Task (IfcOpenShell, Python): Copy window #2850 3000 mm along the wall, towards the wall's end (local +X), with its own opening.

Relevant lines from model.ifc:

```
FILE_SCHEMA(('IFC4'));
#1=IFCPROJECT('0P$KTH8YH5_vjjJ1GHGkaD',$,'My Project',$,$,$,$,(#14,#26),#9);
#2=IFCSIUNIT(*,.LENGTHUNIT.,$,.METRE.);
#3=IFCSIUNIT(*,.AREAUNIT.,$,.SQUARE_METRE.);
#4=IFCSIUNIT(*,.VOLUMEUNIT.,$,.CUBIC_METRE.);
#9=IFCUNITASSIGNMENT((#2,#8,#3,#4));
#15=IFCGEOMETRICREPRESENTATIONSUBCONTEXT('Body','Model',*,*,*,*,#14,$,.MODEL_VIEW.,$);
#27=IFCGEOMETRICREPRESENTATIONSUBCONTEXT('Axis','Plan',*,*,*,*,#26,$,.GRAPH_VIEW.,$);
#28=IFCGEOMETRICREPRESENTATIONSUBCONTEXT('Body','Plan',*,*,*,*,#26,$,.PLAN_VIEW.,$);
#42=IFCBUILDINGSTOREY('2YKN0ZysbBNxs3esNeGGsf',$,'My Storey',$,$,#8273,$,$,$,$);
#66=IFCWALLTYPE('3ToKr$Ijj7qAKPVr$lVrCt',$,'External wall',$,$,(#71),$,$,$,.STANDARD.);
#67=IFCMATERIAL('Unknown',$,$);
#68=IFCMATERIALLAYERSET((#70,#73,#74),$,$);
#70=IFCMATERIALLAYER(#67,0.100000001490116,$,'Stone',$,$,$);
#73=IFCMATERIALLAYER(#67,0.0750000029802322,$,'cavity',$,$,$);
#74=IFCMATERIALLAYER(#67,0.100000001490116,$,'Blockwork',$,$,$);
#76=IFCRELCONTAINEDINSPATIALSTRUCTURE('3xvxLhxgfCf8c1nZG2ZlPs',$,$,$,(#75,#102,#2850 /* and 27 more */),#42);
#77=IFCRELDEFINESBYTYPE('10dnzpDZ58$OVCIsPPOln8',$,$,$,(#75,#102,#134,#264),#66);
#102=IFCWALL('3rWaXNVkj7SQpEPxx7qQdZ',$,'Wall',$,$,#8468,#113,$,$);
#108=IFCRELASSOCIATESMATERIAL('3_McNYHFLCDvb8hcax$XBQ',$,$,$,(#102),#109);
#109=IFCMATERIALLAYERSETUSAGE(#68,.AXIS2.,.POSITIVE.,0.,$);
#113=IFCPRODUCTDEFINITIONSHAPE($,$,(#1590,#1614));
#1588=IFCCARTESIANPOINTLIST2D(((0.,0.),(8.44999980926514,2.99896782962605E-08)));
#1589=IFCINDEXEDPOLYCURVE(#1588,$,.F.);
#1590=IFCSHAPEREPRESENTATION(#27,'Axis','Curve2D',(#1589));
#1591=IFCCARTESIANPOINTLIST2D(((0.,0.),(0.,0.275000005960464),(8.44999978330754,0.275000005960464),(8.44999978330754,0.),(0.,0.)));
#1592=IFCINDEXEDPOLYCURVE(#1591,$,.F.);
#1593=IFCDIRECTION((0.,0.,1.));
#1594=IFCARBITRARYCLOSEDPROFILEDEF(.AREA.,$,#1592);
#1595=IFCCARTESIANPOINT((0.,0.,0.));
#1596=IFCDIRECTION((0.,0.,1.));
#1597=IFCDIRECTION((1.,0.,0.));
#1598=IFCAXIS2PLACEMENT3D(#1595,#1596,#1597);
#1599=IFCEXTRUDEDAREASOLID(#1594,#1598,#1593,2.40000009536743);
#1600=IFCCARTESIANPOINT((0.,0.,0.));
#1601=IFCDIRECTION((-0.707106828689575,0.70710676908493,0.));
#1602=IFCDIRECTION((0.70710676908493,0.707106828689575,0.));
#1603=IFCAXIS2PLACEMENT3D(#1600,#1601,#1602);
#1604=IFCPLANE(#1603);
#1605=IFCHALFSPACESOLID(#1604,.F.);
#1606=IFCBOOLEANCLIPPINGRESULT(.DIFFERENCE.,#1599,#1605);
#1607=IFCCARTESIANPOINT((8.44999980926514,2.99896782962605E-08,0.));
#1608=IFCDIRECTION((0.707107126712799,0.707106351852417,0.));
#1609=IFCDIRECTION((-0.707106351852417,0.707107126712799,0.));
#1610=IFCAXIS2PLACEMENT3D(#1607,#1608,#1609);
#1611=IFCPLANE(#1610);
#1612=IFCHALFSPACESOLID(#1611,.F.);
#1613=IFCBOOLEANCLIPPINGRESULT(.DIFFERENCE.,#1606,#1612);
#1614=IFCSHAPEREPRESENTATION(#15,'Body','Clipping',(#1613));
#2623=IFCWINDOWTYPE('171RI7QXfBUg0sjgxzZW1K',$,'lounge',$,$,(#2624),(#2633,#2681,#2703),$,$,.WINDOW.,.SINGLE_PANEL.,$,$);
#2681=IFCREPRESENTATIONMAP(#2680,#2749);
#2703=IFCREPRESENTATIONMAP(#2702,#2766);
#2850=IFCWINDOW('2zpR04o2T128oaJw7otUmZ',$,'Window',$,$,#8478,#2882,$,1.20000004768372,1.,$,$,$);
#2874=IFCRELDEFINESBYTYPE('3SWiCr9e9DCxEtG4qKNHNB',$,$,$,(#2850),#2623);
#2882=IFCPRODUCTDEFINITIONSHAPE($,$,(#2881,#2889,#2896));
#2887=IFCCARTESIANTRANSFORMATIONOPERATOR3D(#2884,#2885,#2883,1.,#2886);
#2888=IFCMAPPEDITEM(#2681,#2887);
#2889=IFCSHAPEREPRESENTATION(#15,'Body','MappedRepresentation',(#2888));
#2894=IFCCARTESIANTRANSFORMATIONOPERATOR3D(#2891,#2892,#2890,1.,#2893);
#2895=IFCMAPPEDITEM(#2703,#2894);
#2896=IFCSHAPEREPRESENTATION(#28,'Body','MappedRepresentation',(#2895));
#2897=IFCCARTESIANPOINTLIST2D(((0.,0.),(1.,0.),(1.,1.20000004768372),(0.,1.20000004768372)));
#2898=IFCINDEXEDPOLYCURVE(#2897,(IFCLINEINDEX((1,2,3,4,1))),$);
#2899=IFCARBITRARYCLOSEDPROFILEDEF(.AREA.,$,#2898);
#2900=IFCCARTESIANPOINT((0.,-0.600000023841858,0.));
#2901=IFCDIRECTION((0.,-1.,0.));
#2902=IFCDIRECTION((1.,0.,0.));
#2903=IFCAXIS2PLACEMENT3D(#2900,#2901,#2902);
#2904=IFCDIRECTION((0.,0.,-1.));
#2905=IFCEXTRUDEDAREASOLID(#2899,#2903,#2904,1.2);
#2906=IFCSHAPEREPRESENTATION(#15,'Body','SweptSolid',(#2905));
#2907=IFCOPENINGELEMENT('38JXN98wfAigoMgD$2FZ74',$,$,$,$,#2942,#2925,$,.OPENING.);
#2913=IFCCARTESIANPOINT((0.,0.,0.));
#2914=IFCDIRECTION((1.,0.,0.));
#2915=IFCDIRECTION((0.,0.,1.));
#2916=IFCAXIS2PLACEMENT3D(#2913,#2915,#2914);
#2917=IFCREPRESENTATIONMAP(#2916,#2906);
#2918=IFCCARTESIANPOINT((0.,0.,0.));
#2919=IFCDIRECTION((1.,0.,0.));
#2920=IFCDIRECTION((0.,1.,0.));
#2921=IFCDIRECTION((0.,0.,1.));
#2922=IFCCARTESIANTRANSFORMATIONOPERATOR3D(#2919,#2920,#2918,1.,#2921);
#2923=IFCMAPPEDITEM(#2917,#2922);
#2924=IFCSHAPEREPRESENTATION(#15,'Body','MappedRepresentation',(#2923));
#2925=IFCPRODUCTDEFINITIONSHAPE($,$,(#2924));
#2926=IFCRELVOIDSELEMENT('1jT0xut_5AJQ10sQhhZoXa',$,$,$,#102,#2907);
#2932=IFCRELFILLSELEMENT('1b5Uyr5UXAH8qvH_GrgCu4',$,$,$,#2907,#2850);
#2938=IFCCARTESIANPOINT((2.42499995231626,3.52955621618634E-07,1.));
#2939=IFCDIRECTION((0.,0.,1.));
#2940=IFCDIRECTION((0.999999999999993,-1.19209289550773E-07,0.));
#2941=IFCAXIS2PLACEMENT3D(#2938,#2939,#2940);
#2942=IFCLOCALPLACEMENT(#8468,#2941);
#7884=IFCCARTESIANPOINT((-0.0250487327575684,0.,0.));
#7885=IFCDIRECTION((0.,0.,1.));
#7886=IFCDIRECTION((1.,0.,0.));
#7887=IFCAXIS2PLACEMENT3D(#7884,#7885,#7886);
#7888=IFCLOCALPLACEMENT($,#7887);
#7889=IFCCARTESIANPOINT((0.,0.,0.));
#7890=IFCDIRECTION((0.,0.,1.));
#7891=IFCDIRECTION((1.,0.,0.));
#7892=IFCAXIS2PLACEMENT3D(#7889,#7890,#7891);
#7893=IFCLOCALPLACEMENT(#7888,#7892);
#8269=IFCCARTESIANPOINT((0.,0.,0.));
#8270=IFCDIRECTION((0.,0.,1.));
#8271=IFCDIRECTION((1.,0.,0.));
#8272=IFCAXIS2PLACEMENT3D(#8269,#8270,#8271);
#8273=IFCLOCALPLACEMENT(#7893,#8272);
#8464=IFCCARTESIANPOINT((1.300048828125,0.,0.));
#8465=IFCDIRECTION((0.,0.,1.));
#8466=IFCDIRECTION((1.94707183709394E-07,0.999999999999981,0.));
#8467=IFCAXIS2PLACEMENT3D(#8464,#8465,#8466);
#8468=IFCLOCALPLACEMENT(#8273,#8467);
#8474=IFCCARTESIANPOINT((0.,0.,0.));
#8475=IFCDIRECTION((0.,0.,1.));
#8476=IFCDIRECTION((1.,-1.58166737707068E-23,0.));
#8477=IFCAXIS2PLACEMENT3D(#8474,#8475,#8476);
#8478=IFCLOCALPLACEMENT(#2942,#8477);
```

```python
import ifcopenshell
import ifcopenshell.api.feature
import ifcopenshell.api.geometry
import ifcopenshell.api.root
import ifcopenshell.geom
import ifcopenshell.util.element
import ifcopenshell.util.placement
import ifcopenshell.util.shape

model = ifcopenshell.open("model.ifc")
settings = ifcopenshell.geom.settings()


def volume(element):
    """Net volume in cubic metres, openings subtracted."""
    shape = ifcopenshell.geom.create_shape(settings, element)
    return ifcopenshell.util.shape.get_volume(shape.geometry)


window = model.by_guid("2zpR04o2T128oaJw7otUmZ")
opening = window.FillsVoids[0].RelatingOpeningElement
wall = opening.VoidsElements[0].RelatingBuildingElement
before = volume(wall)
shift = ifcopenshell.util.placement.get_local_placement(wall.ObjectPlacement)[:3, 0] * 3.0

# copy_class copies the void relationship, type, container and properties, but no geometry.
new_opening = ifcopenshell.api.root.copy_class(model, product=opening)
new_opening.Representation = ifcopenshell.util.element.copy_deep(
    model, opening.Representation, exclude=["IfcGeometricRepresentationContext", "IfcRepresentationMap"]
)
new_window = ifcopenshell.api.root.copy_class(model, product=window)
new_window.Representation = ifcopenshell.util.element.copy_deep(
    model, window.Representation, exclude=["IfcGeometricRepresentationContext", "IfcRepresentationMap"]
)
ifcopenshell.api.feature.add_filling(model, opening=new_opening, element=new_window)

for old, new in ((opening, new_opening), (window, new_window)):
    matrix = ifcopenshell.util.placement.get_local_placement(old.ObjectPlacement)
    matrix[:3, 3] += shift
    ifcopenshell.api.geometry.edit_object_placement(model, product=new, matrix=matrix, is_si=False)

after = volume(wall)

print(f"wall volume {before:.3f} -> {after:.3f} m3")

model.write("model_v2.ifc")
```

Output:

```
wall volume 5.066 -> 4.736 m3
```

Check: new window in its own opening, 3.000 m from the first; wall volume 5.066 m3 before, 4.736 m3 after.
